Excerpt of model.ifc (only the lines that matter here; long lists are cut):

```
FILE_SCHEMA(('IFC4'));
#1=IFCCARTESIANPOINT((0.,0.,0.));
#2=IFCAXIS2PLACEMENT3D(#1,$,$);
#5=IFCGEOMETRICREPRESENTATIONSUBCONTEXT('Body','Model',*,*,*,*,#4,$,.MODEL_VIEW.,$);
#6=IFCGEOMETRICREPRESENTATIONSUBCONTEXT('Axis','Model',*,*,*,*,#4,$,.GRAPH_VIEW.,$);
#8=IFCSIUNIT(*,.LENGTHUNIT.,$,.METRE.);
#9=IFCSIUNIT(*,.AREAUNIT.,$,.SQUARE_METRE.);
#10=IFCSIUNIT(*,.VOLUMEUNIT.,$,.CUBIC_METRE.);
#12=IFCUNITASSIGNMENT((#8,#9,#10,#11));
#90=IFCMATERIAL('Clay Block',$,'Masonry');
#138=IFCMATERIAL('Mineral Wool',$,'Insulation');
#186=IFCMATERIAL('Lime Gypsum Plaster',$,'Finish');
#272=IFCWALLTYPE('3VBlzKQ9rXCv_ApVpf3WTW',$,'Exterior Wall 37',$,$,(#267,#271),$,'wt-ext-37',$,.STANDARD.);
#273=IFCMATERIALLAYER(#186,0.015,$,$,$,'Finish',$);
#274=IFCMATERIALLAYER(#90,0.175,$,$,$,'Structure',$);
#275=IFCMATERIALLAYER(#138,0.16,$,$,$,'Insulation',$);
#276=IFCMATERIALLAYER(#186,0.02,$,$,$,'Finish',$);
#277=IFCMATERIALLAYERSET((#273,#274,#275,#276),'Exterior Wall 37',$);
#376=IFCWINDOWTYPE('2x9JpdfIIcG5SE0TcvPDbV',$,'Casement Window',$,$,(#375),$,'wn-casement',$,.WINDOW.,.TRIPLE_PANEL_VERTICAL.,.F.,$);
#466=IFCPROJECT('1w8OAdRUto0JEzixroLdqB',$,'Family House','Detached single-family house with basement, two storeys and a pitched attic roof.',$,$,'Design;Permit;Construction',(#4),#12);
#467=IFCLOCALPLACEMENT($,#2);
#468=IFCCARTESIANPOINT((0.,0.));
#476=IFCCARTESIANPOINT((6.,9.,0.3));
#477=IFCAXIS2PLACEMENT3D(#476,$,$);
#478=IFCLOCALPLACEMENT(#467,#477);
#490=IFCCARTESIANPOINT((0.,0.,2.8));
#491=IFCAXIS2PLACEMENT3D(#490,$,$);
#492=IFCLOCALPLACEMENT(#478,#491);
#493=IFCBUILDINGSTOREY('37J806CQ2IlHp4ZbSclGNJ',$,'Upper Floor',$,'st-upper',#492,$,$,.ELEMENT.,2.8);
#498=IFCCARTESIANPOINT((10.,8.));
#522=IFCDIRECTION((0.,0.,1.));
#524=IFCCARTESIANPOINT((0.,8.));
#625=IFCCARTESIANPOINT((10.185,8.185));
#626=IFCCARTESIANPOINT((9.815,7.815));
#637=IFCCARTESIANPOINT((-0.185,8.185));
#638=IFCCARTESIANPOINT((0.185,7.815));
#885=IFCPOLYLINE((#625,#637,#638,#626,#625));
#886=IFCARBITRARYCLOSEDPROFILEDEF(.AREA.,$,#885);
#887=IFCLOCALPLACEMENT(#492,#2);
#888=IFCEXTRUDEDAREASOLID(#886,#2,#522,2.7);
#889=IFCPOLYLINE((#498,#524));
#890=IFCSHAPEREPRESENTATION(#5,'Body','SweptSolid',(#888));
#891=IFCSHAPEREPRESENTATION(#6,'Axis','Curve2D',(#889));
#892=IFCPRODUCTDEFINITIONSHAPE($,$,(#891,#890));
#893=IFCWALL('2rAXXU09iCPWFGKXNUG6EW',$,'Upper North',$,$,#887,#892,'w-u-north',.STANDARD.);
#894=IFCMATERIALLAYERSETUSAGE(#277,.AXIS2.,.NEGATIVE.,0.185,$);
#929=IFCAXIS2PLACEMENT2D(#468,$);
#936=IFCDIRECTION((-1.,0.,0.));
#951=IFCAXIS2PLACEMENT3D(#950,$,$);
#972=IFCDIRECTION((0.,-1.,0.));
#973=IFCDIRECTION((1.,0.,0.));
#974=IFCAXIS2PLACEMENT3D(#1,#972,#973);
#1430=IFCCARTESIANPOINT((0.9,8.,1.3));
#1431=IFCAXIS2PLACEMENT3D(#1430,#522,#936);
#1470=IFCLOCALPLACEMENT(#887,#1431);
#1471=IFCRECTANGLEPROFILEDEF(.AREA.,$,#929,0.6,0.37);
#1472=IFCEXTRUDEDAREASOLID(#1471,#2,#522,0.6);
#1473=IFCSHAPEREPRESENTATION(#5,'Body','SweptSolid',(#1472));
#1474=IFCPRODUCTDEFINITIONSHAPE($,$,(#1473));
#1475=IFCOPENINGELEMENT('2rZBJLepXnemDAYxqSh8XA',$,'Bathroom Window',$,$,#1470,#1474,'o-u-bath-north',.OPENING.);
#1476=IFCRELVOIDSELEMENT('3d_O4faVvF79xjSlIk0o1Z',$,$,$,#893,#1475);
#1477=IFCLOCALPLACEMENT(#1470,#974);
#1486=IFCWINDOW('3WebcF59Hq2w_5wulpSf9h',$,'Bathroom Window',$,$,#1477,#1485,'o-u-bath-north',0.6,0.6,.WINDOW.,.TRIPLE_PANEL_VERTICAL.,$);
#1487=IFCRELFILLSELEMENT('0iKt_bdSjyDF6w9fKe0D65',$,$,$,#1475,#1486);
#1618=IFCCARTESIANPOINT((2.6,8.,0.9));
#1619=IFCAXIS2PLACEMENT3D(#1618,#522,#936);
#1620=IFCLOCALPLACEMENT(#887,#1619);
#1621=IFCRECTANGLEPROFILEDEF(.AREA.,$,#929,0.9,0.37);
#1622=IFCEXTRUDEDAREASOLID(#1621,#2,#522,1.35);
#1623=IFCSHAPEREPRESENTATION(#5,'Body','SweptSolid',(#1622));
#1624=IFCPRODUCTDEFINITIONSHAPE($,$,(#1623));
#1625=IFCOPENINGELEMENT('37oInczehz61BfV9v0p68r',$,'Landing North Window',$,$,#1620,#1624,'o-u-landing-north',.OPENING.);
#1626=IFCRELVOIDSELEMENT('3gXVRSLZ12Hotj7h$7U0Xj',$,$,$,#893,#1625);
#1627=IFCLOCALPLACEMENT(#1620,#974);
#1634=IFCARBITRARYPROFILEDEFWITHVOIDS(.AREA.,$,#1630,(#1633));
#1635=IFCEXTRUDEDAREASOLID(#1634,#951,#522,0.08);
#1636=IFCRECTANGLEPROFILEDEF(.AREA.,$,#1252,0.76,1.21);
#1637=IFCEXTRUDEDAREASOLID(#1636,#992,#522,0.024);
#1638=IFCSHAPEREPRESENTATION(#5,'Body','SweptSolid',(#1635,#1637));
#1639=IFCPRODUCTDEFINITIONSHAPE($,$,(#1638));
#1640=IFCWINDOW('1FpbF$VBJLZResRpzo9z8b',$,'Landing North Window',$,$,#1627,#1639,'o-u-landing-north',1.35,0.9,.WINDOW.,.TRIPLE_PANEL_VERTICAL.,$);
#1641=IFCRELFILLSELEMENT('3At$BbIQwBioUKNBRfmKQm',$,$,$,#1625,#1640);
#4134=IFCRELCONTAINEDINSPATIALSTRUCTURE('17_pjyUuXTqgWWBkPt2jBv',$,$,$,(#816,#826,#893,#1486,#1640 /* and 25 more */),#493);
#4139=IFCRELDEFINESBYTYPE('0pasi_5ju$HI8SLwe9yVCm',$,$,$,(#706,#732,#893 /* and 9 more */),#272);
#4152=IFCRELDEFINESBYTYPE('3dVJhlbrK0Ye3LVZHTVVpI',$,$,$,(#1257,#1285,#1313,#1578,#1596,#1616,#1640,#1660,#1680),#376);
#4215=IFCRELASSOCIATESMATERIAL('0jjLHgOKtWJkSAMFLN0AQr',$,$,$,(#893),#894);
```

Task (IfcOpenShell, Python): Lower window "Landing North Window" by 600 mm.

```python
import numpy as np
import ifcopenshell
import ifcopenshell.api.geometry
import ifcopenshell.util.placement
import ifcopenshell.util.unit

model = ifcopenshell.open("model.ifc")
unit_scale = ifcopenshell.util.unit.calculate_unit_scale(model)

window = model.by_guid("1FpbF$VBJLZResRpzo9z8b")
opening = window.FillsVoids[0].RelatingOpeningElement
dz = -0.6

shift = np.array([0.0, 0.0, dz])
# The window is placed relative to its opening, so it follows when the opening moves.
matrix = ifcopenshell.util.placement.get_local_placement(opening.ObjectPlacement)
matrix[:3, 3] += shift
ifcopenshell.api.geometry.edit_object_placement(
    model, product=opening, matrix=matrix, is_si=False, should_transform_children=True
)

print(f"moved by {dz * unit_scale:+.3f} m")

model.write("model_v2.ifc")
```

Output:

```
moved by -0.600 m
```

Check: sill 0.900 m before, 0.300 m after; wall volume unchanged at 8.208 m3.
